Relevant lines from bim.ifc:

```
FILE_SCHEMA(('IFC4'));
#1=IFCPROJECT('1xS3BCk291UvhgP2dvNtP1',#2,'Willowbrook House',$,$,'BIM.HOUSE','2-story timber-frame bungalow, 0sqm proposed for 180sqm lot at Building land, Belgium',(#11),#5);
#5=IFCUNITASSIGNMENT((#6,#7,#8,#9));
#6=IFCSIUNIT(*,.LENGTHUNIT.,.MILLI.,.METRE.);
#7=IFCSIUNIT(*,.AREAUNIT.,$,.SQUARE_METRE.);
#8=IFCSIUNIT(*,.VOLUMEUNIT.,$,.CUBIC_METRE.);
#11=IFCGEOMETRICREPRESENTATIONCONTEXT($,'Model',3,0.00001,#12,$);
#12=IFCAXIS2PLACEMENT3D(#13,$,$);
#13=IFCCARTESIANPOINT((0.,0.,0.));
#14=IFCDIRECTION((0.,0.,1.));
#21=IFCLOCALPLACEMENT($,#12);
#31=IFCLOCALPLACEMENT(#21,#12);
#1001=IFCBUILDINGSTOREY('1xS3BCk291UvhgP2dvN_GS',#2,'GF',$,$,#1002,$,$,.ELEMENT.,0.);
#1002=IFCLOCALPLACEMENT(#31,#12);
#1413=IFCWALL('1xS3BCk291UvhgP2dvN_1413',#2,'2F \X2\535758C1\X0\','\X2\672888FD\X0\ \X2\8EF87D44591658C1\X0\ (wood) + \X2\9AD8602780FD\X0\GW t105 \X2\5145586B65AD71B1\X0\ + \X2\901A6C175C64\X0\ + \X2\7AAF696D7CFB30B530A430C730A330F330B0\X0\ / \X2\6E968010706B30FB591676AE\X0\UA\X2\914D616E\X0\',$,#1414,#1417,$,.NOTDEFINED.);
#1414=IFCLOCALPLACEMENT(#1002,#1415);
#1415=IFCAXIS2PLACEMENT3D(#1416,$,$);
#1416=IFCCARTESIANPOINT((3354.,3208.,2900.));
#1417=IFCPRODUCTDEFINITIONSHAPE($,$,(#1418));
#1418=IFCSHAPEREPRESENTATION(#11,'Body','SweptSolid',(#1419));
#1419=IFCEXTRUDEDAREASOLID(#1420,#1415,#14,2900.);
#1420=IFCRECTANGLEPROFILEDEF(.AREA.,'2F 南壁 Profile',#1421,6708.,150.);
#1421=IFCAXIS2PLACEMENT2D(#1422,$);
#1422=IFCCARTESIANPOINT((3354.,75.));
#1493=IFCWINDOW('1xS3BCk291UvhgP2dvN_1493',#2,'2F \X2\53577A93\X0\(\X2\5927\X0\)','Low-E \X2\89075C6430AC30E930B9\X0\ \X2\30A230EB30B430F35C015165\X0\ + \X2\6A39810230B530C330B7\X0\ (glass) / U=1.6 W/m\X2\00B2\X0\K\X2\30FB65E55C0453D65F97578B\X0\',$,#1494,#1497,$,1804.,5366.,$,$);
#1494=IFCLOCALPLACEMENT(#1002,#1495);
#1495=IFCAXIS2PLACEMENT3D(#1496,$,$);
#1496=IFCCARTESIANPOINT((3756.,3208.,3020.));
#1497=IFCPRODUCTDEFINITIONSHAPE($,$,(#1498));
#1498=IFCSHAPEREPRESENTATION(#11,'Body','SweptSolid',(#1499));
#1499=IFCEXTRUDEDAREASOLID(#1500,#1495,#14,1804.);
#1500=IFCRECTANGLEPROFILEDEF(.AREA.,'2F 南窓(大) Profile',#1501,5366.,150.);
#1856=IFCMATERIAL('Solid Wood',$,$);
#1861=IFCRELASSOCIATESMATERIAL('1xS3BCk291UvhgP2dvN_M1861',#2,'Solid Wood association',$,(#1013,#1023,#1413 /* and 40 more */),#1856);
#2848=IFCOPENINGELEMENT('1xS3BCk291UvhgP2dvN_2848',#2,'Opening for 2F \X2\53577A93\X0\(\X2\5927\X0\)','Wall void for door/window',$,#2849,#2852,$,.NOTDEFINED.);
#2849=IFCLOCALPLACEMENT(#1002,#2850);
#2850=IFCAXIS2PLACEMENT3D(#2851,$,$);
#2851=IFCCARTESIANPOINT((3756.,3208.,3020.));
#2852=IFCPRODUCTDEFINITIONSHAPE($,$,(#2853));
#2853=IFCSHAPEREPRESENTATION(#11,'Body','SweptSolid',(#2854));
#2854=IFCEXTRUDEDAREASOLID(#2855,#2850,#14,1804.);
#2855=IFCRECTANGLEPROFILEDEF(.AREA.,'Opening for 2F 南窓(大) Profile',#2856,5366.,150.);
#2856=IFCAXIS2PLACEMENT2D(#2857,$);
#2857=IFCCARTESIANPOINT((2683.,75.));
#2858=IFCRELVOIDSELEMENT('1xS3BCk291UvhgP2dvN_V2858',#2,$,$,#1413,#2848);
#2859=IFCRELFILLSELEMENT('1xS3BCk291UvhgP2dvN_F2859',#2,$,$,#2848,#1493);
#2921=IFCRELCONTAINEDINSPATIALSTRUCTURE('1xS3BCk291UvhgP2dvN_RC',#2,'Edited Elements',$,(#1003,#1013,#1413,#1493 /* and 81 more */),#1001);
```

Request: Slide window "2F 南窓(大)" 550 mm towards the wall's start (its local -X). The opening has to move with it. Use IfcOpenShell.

```python
import ifcopenshell
import ifcopenshell.api.geometry
import ifcopenshell.util.placement

model = ifcopenshell.open("bim.ifc")

window = model.by_id(1493)
opening = window.FillsVoids[0].RelatingOpeningElement
wall = opening.VoidsElements[0].RelatingBuildingElement

wall_matrix = ifcopenshell.util.placement.get_local_placement(wall.ObjectPlacement)
shift = wall_matrix[:3, 0] * -550.0
before = ifcopenshell.util.placement.get_local_placement(window.ObjectPlacement)[:3, 3].copy()

# The window is not placed relative to its opening, so move both.
for product in (opening, window):
    matrix = ifcopenshell.util.placement.get_local_placement(product.ObjectPlacement)
    matrix[:3, 3] += shift
    ifcopenshell.api.geometry.edit_object_placement(model, product=product, matrix=matrix, is_si=False)

after = ifcopenshell.util.placement.get_local_placement(window.ObjectPlacement)[:3, 3]
print("window moved by", (after - before).round(3) + 0.0)

model.write("bim-out.ifc")
```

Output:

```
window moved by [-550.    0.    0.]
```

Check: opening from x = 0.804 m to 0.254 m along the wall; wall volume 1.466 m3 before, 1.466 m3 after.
